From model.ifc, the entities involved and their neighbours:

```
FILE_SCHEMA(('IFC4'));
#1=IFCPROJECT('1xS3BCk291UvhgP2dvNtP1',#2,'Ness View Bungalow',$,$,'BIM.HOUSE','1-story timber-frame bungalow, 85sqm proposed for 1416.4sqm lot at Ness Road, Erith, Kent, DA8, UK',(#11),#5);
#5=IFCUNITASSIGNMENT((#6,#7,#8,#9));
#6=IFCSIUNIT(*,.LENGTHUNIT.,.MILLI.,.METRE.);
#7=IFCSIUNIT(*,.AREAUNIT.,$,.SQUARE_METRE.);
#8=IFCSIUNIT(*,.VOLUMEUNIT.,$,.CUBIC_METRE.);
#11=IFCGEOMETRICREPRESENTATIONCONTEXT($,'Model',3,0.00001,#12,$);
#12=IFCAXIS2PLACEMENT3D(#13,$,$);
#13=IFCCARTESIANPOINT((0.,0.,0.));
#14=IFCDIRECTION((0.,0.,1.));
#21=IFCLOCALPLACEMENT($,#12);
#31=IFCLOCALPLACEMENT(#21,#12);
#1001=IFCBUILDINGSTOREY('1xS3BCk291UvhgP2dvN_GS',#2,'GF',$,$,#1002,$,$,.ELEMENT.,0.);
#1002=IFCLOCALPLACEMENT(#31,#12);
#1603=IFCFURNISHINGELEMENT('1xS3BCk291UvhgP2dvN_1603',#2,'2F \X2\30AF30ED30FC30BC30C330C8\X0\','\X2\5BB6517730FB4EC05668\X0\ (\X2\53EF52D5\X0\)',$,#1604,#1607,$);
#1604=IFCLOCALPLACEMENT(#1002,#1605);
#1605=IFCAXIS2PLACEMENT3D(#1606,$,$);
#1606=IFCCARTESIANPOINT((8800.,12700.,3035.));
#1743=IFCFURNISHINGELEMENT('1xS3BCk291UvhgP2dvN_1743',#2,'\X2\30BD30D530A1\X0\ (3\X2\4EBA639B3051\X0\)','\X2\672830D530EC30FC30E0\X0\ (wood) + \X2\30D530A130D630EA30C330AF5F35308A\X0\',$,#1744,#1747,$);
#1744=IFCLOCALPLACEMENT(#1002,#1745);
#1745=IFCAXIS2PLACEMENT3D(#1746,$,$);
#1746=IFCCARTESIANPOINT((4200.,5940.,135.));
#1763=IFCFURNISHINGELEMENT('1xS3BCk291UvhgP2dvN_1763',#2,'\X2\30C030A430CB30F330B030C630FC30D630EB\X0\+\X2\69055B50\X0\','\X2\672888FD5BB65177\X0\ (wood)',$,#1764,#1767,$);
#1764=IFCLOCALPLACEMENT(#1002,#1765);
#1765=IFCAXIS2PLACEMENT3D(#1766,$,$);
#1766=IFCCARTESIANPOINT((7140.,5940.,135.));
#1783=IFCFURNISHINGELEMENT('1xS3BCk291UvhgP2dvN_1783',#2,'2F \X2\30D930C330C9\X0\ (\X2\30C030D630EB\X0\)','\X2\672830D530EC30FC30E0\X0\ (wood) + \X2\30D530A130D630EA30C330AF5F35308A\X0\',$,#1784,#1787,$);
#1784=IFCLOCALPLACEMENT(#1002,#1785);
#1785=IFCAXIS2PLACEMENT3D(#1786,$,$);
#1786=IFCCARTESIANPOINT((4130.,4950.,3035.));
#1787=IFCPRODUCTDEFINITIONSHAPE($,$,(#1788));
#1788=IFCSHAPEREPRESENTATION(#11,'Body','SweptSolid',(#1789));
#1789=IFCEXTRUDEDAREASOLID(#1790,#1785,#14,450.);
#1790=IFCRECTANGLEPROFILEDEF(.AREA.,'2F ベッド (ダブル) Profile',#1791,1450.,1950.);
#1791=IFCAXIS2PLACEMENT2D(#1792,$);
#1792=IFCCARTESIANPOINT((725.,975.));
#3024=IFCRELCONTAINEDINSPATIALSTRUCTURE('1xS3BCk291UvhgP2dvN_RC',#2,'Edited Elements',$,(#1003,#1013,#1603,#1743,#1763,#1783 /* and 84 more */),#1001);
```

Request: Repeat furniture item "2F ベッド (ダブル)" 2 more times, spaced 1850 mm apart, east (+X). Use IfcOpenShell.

```python
import numpy as np
import ifcopenshell
import ifcopenshell.api.geometry
import ifcopenshell.api.root
import ifcopenshell.util.element
import ifcopenshell.util.placement

model = ifcopenshell.open("model.ifc")


def reuse_history(source, copy):
    """copy_class also copies each property set's owner history, people and application; keep the originals."""
    for rel in copy.IsDefinedBy:
        if rel.is_a("IfcRelDefinesByProperties") and (history := rel.RelatingPropertyDefinition.OwnerHistory):
            rel.RelatingPropertyDefinition.OwnerHistory = source.OwnerHistory
            ifcopenshell.util.element.remove_deep2(model, history)


source = model.by_id(1783)
base = ifcopenshell.util.placement.get_local_placement(source.ObjectPlacement)
step = np.array([1.0, 0.0, 0.0]) * 1850.0

for i in range(1, 3):
    copy = ifcopenshell.api.root.copy_class(model, product=source)
    copy.Representation = ifcopenshell.util.element.copy_deep(
        model, source.Representation, exclude=["IfcGeometricRepresentationContext", "IfcRepresentationMap"]
    )
    reuse_history(source, copy)
    matrix = base.copy()
    matrix[:3, 3] += i * step
    print("added at", matrix[:3, 3].round(3) + 0.0)
    ifcopenshell.api.geometry.edit_object_placement(model, product=copy, matrix=matrix, is_si=False)

model.write("model_rev.ifc")
```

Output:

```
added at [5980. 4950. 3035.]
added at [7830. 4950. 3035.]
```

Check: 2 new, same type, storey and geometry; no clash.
